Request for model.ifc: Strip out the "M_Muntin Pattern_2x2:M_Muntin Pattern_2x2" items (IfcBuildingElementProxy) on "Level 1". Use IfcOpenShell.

First a look at what the model holds.

```python
import ifcopenshell
import ifcopenshell.util.element

model = ifcopenshell.open("model.ifc")
print(model.schema)
storey = next(s for s in model.by_type("IfcBuildingStorey") if s.Name == "Level 1")
proxies = [e for e in ifcopenshell.util.element.get_decomposition(storey) if e.is_a("IfcBuildingElementProxy")]
seen = {}
for e in proxies:
    element_type = ifcopenshell.util.element.get_type(e)
    name = element_type.Name if element_type not in (None, e) else None
    seen[name] = seen.get(name, 0) + 1
for name, count in sorted(seen.items(), key=str):
    print(count, "x", name)
```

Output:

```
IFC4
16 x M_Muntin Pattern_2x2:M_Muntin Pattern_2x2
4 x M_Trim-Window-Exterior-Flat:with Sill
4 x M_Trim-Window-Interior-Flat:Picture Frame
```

```python
import ifcopenshell
import ifcopenshell.api.root
import ifcopenshell.util.element

model = ifcopenshell.open("model.ifc")

storey = next(s for s in model.by_type("IfcBuildingStorey") if s.Name == "Level 1")
proxies = [e for e in ifcopenshell.util.element.get_decomposition(storey) if e.is_a("IfcBuildingElementProxy")]
targets = [e for e in proxies if (t := ifcopenshell.util.element.get_type(e)) not in (None, e) and t.Name == "M_Muntin Pattern_2x2:M_Muntin Pattern_2x2"]

for e in targets:
    ifcopenshell.api.root.remove_product(model, product=e)
print(len(targets), "removed")

model.write("model_v2.ifc")
```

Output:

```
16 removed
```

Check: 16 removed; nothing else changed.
